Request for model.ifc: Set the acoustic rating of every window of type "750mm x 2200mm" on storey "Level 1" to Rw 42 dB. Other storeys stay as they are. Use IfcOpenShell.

First a look at what the model holds.

```python
import ifcopenshell
import ifcopenshell.util.element

model = ifcopenshell.open("model.ifc")
print(model.schema)
storey = next(s for s in model.by_type("IfcBuildingStorey") if s.Name == "Level 1")
windows = [e for e in ifcopenshell.util.element.get_decomposition(storey) if e.is_a("IfcWindow")]
seen = {}
for e in windows:
    element_type = ifcopenshell.util.element.get_type(e)
    key = (element_type.Name if element_type != e and element_type else None, ifcopenshell.util.element.get_pset(e, "Pset_WindowCommon", "AcousticRating"))
    seen[key] = seen.get(key, 0) + 1
for (name, value), count in sorted(seen.items(), key=str):
    print(count, "x", name, "|", value)
```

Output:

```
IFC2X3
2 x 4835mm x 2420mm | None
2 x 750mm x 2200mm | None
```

```python
import ifcopenshell
import ifcopenshell.api.pset
import ifcopenshell.util.element

model = ifcopenshell.open("model.ifc")

storey = next(s for s in model.by_type("IfcBuildingStorey") if s.Name == "Level 1")
windows = [e for e in ifcopenshell.util.element.get_decomposition(storey) if e.is_a("IfcWindow")]

count = 0
for e in windows:
    element_type = ifcopenshell.util.element.get_type(e)
    if element_type in (None, e) or element_type.Name != "750mm x 2200mm":
        continue
    # add_pset returns the element's existing set when there is one.
    pset = ifcopenshell.api.pset.add_pset(model, product=e, name="Pset_WindowCommon")
    ifcopenshell.api.pset.edit_pset(model, pset=pset, properties={"AcousticRating": "Rw 42 dB"})
    count += 1

print(count, "windows updated")

model.write("model-out.ifc")
```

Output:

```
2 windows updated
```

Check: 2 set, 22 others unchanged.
